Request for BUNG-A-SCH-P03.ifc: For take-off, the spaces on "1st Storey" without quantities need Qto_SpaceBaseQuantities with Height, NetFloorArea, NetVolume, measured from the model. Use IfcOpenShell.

First a look at what the model holds.

```python
import ifcopenshell
import ifcopenshell.util.element
import ifcopenshell.util.unit

model = ifcopenshell.open("BUNG-A-SCH-P03.ifc")
print(model.schema)
for unit_type in ("LENGTHUNIT", "AREAUNIT", "VOLUMEUNIT"):
    print(unit_type, ifcopenshell.util.unit.calculate_unit_scale(model, unit_type))
storey = next(s for s in model.by_type("IfcBuildingStorey") if s.Name == "1st Storey")
spaces = [e for e in ifcopenshell.util.element.get_decomposition(storey) if e.is_a("IfcSpace")]
for e in sorted(spaces, key=lambda e: e.id()):
    print(e.id(), e.is_a(), e.Name, list(ifcopenshell.util.element.get_psets(e, qtos_only=True)), sep=" | ")
```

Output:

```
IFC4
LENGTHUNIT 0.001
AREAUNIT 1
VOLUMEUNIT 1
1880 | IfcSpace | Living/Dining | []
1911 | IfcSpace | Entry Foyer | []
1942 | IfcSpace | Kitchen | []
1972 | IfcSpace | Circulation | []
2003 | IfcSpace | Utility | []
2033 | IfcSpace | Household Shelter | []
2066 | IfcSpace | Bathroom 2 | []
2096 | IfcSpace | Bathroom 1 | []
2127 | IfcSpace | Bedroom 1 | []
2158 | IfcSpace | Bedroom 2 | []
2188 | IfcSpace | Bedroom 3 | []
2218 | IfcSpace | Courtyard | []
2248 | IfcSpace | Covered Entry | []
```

```python
import ifcopenshell
import ifcopenshell.api.pset
import ifcopenshell.geom
import ifcopenshell.util.element
import ifcopenshell.util.shape
import ifcopenshell.util.unit

model = ifcopenshell.open("BUNG-A-SCH-P03.ifc")
unit_scale = ifcopenshell.util.unit.calculate_unit_scale(model)
area_scale = ifcopenshell.util.unit.calculate_unit_scale(model, "AREAUNIT")
volume_scale = ifcopenshell.util.unit.calculate_unit_scale(model, "VOLUMEUNIT")
settings = ifcopenshell.geom.settings()

storey = next(s for s in model.by_type("IfcBuildingStorey") if s.Name == "1st Storey")
spaces = [e for e in ifcopenshell.util.element.get_decomposition(storey) if e.is_a("IfcSpace")]

for e in sorted(spaces, key=lambda e: e.id()):
    if ifcopenshell.util.element.get_psets(e, qtos_only=True, should_inherit=False):
        continue
    # Geometry comes back in metres, in the element's own axes.
    shape = ifcopenshell.geom.create_shape(settings, e)
    values = {
        "Height": ifcopenshell.util.shape.get_z(shape.geometry) / unit_scale,
        "NetFloorArea": ifcopenshell.util.shape.get_footprint_area(shape.geometry) / area_scale,
        "NetVolume": ifcopenshell.util.shape.get_volume(shape.geometry) / volume_scale,
    }
    qto = ifcopenshell.api.pset.add_qto(model, product=e, name="Qto_SpaceBaseQuantities")
    ifcopenshell.api.pset.edit_qto(model, qto=qto, properties=values)
    print(e.id(), {k: round(v, 3) for k, v in values.items()})

model.write("BUNG-A-SCH-P03_v2.ifc")
```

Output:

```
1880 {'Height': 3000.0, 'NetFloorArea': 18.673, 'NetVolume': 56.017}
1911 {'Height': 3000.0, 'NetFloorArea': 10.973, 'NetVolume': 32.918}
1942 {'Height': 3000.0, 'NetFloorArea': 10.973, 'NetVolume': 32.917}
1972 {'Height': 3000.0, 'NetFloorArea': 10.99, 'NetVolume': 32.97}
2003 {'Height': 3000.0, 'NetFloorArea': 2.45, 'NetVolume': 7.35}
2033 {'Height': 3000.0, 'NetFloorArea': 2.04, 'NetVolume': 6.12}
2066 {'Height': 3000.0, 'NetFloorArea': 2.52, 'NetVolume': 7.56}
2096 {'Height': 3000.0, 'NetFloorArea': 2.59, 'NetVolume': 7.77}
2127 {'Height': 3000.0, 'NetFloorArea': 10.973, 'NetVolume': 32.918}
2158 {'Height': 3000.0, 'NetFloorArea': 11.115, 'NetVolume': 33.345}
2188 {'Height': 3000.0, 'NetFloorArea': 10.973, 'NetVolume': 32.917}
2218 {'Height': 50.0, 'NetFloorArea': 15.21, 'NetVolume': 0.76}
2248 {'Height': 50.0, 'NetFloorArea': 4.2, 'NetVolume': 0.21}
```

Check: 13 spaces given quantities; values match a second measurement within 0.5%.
